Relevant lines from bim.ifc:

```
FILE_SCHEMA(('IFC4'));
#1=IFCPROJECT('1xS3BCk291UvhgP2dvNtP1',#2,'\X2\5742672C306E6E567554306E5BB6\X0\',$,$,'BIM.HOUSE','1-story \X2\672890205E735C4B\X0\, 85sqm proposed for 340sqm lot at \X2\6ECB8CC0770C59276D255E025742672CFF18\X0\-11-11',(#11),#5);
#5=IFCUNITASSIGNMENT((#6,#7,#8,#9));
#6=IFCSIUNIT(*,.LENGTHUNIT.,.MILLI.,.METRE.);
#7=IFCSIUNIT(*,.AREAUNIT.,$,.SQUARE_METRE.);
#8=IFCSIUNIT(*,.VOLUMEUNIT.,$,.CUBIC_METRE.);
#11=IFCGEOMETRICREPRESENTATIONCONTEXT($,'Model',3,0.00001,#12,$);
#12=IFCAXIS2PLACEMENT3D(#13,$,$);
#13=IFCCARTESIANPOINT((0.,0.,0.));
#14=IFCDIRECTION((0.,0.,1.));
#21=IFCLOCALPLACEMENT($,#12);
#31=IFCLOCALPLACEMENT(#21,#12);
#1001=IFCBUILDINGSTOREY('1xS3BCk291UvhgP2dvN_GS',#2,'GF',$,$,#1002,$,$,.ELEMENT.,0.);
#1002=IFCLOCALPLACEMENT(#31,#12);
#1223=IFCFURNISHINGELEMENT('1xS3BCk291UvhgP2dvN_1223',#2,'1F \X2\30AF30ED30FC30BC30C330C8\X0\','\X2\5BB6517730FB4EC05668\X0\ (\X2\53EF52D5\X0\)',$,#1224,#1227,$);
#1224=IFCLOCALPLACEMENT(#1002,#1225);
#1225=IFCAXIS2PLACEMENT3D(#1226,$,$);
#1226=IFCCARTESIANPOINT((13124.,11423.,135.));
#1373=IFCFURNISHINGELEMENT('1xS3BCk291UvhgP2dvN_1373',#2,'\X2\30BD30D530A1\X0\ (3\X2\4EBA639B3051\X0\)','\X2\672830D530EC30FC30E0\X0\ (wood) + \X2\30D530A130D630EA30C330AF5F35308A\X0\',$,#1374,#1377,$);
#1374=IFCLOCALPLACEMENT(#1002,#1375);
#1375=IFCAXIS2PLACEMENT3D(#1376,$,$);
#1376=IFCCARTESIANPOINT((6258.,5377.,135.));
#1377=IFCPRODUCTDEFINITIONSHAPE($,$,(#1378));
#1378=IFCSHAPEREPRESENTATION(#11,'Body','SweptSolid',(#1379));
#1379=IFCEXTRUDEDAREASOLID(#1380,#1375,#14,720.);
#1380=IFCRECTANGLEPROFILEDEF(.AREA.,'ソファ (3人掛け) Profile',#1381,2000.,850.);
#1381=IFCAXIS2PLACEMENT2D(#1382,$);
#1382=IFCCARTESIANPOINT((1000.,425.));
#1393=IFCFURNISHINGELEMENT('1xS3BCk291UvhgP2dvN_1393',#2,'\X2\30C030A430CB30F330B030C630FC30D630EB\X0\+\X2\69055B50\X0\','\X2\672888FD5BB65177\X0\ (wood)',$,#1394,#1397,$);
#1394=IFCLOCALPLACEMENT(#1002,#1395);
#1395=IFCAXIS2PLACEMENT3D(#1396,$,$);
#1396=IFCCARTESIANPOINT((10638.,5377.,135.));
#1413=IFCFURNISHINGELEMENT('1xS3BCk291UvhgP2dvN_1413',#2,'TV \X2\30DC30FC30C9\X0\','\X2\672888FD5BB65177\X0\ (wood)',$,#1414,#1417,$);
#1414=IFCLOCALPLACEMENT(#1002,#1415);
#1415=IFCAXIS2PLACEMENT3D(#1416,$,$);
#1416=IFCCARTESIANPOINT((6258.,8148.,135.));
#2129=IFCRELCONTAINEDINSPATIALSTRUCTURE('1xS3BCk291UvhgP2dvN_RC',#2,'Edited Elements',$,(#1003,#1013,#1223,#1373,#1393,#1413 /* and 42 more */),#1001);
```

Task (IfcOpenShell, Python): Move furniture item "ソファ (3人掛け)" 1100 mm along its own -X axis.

```python
import ifcopenshell
import ifcopenshell.api.geometry
import ifcopenshell.util.placement

model = ifcopenshell.open("bim.ifc")

item = model.by_guid("1xS3BCk291UvhgP2dvN_1373")
matrix = ifcopenshell.util.placement.get_local_placement(item.ObjectPlacement)
matrix[:3, 3] -= matrix[:3, 0] * 1100.0
ifcopenshell.api.geometry.edit_object_placement(model, product=item, matrix=matrix, is_si=False)

print(ifcopenshell.util.placement.get_local_placement(item.ObjectPlacement).round(3) + 0.0)

model.write("bim_edited.ifc")
```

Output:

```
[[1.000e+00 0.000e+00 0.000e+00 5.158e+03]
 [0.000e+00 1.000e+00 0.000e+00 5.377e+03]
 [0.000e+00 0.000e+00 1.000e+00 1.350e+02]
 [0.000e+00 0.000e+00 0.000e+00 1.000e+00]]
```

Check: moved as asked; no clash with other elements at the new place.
